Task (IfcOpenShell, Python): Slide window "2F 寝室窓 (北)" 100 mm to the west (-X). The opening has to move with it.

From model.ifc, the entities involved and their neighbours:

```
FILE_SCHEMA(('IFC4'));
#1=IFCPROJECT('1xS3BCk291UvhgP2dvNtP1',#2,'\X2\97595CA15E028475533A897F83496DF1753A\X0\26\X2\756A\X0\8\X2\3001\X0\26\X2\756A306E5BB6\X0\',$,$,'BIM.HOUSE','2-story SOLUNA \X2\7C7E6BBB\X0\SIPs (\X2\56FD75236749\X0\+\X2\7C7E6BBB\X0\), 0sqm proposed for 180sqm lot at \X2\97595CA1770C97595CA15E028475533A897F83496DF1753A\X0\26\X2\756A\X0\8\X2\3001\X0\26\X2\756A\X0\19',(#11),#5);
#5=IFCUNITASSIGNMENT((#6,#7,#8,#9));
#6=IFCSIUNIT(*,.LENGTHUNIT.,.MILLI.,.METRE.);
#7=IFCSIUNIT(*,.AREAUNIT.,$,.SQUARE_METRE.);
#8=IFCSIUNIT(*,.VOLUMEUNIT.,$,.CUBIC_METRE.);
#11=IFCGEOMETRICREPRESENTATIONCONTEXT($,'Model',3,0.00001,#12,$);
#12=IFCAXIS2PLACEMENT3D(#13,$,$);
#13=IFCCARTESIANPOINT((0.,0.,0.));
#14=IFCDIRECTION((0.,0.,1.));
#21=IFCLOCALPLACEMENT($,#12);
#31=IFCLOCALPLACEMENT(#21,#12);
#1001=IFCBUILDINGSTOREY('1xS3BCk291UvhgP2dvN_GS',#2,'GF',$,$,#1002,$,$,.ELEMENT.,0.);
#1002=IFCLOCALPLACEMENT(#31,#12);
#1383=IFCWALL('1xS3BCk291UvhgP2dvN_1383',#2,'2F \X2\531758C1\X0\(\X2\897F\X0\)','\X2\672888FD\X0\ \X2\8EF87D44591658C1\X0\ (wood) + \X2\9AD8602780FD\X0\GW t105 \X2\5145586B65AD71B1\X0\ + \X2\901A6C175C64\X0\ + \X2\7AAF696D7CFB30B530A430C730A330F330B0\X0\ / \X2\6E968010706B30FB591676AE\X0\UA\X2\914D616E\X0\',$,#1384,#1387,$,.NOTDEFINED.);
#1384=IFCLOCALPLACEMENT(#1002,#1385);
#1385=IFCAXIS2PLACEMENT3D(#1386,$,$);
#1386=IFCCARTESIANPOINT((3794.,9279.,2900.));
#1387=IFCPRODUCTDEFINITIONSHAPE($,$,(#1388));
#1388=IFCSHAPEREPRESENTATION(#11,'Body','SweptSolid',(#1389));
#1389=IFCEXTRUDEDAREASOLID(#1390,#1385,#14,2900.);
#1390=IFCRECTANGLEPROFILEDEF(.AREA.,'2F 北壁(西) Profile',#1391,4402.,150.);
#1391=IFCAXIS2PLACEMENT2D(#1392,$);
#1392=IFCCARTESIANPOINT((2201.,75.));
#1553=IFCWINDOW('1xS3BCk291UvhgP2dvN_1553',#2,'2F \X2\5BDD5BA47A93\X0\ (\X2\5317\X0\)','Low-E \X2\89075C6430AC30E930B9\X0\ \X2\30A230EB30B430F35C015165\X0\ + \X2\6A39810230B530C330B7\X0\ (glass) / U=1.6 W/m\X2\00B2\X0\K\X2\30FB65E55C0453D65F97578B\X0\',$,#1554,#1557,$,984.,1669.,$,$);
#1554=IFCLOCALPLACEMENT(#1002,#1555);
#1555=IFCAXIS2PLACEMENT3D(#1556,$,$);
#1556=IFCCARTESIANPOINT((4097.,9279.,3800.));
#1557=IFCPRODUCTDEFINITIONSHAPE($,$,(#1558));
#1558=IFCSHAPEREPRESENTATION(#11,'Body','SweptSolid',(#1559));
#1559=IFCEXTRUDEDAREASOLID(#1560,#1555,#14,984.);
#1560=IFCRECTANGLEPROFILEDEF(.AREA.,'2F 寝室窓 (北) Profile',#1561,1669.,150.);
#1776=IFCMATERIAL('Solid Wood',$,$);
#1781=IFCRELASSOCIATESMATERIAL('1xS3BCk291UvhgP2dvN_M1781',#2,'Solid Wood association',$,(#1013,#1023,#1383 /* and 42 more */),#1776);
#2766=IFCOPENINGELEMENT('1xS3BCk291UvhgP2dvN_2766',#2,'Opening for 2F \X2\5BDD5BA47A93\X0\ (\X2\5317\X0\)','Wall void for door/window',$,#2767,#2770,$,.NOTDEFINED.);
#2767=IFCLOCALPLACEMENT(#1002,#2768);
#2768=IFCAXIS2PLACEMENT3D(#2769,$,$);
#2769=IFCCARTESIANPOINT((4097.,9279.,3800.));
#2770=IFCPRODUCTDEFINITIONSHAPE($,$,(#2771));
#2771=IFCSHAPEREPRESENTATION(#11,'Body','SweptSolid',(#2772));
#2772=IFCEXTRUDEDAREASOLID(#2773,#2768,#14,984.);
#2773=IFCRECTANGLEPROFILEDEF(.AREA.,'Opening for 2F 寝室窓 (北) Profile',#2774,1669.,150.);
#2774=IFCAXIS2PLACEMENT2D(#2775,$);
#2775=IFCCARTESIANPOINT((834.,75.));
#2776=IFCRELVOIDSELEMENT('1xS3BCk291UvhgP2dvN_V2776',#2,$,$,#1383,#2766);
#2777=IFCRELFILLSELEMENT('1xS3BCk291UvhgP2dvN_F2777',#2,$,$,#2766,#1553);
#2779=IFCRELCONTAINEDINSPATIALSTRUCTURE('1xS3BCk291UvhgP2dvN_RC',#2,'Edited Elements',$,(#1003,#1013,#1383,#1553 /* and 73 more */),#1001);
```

```python
import ifcopenshell
import ifcopenshell.api.geometry
import ifcopenshell.util.placement
import ifcopenshell.util.unit

model = ifcopenshell.open("model.ifc")
unit_scale = ifcopenshell.util.unit.calculate_unit_scale(model)

window = model.by_guid("1xS3BCk291UvhgP2dvN_1553")
opening = window.FillsVoids[0].RelatingOpeningElement
wall = opening.VoidsElements[0].RelatingBuildingElement

wall_matrix = ifcopenshell.util.placement.get_local_placement(wall.ObjectPlacement)
shift = wall_matrix[:3, 0] * -0.1 / unit_scale
before = ifcopenshell.util.placement.get_local_placement(window.ObjectPlacement)[:3, 3].copy()

# The window is not placed relative to its opening, so move both.
for product in (opening, window):
    matrix = ifcopenshell.util.placement.get_local_placement(product.ObjectPlacement)
    matrix[:3, 3] += shift
    ifcopenshell.api.geometry.edit_object_placement(model, product=product, matrix=matrix, is_si=False)

after = ifcopenshell.util.placement.get_local_placement(window.ObjectPlacement)[:3, 3]
print("window moved by", (after - before).round(3) + 0.0)

model.write("model_rev.ifc")
```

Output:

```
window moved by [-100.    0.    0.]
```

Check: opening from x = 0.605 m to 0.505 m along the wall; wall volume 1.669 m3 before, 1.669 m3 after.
